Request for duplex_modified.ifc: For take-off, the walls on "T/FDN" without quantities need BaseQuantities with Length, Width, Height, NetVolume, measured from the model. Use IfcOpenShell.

First a look at what the model holds.

```python
import ifcopenshell
import ifcopenshell.util.element
import ifcopenshell.util.unit

model = ifcopenshell.open("duplex_modified.ifc")
print(model.schema)
for unit_type in ("LENGTHUNIT", "AREAUNIT", "VOLUMEUNIT"):
    print(unit_type, ifcopenshell.util.unit.calculate_unit_scale(model, unit_type))
storey = next(s for s in model.by_type("IfcBuildingStorey") if s.Name == "T/FDN")
walls = [e for e in ifcopenshell.util.element.get_decomposition(storey) if e.is_a("IfcWall")]
for e in sorted(walls, key=lambda e: e.id()):
    print(e.id(), e.is_a(), e.Name, list(ifcopenshell.util.element.get_psets(e, qtos_only=True)), sep=" | ")
```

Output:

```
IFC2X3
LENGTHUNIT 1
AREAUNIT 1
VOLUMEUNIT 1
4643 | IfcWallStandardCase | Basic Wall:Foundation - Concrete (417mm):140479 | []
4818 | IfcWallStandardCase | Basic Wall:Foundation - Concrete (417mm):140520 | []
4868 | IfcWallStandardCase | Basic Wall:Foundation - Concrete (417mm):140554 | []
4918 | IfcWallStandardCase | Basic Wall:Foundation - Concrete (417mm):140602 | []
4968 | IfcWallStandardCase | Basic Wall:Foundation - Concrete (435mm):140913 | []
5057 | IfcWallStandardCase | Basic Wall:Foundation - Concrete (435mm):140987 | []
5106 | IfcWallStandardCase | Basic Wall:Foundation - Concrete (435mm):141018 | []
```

```python
import ifcopenshell
import ifcopenshell.api.pset
import ifcopenshell.geom
import ifcopenshell.util.element
import ifcopenshell.util.shape
import ifcopenshell.util.unit

model = ifcopenshell.open("duplex_modified.ifc")
unit_scale = ifcopenshell.util.unit.calculate_unit_scale(model)
volume_scale = ifcopenshell.util.unit.calculate_unit_scale(model, "VOLUMEUNIT")
settings = ifcopenshell.geom.settings()

storey = next(s for s in model.by_type("IfcBuildingStorey") if s.Name == "T/FDN")
walls = [e for e in ifcopenshell.util.element.get_decomposition(storey) if e.is_a("IfcWall")]

for e in sorted(walls, key=lambda e: e.id()):
    if ifcopenshell.util.element.get_psets(e, qtos_only=True, should_inherit=False):
        continue
    # Geometry comes back in metres, in the element's own axes.
    shape = ifcopenshell.geom.create_shape(settings, e)
    values = {
        "Length": ifcopenshell.util.shape.get_x(shape.geometry) / unit_scale,
        "Width": ifcopenshell.util.shape.get_y(shape.geometry) / unit_scale,
        "Height": ifcopenshell.util.shape.get_z(shape.geometry) / unit_scale,
        "NetVolume": ifcopenshell.util.shape.get_volume(shape.geometry) / volume_scale,
    }
    qto = ifcopenshell.api.pset.add_qto(model, product=e, name="BaseQuantities")
    ifcopenshell.api.pset.edit_qto(model, qto=qto, properties=values)
    print(e.id(), {k: round(v, 3) for k, v in values.items()})

model.write("duplex_modified_v2.ifc")
```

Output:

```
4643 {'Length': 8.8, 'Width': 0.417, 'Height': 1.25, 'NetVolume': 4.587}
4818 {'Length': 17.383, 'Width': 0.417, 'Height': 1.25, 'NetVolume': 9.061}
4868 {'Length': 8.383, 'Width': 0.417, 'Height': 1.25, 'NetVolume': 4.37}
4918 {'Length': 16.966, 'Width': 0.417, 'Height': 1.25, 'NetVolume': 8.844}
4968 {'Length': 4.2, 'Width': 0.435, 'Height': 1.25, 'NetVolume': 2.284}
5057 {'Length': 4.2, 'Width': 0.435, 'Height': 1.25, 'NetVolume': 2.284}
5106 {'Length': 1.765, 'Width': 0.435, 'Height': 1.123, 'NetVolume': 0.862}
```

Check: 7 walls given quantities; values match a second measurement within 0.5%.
